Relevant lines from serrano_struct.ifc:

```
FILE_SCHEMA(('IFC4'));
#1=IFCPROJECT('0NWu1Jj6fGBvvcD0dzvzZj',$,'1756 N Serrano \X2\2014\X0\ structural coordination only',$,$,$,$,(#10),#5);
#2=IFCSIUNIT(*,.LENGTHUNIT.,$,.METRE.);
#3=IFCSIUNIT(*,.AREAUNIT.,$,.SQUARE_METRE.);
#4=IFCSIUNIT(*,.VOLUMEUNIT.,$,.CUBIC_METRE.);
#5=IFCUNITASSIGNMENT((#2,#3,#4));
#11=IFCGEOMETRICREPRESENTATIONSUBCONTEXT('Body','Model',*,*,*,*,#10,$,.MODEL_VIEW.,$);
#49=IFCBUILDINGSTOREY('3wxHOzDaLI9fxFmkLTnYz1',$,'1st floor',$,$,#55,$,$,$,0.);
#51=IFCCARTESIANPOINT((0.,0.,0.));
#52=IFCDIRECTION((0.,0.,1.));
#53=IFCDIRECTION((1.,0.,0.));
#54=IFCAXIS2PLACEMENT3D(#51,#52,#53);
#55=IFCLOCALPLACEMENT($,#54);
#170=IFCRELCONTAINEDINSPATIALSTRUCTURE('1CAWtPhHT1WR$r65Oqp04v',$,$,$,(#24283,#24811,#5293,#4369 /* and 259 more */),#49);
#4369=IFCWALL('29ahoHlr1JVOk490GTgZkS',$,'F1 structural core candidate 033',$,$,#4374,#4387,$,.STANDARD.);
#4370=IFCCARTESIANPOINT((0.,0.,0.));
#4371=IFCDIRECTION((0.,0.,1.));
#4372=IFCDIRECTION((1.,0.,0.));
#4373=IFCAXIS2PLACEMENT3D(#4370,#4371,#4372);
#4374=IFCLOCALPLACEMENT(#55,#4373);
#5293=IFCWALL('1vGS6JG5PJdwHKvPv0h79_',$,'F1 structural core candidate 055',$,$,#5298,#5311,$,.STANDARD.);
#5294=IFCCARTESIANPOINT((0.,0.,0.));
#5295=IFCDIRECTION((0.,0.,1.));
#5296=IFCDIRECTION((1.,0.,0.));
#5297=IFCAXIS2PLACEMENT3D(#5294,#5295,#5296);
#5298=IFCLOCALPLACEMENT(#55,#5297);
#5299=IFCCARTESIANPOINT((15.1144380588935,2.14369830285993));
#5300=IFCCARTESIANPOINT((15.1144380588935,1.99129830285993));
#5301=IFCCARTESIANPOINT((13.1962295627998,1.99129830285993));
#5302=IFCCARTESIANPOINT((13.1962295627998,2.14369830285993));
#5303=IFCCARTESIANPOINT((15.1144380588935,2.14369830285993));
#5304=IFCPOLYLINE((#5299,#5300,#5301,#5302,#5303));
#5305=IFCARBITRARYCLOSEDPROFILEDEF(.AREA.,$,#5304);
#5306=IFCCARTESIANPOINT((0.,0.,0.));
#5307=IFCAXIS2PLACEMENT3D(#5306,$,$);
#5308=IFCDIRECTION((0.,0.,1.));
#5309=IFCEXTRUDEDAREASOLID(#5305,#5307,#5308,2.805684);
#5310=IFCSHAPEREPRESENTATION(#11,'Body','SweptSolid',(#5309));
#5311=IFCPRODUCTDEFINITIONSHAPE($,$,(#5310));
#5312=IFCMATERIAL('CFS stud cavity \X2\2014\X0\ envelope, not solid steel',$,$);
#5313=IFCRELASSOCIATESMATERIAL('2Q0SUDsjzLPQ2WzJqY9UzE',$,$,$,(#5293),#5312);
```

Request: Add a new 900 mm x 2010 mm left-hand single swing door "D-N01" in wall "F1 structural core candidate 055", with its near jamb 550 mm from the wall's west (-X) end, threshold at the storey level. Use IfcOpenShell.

```python
import numpy as np
import ifcopenshell
import ifcopenshell.api.feature
import ifcopenshell.api.geometry
import ifcopenshell.api.root
import ifcopenshell.api.spatial
import ifcopenshell.geom
import ifcopenshell.util.element
import ifcopenshell.util.placement
import ifcopenshell.util.representation
import ifcopenshell.util.shape
import ifcopenshell.util.unit

model = ifcopenshell.open("serrano_struct.ifc")
unit_scale = ifcopenshell.util.unit.calculate_unit_scale(model)
settings = ifcopenshell.geom.settings()


def volume(element):
    """Net volume in cubic metres, openings subtracted."""
    shape = ifcopenshell.geom.create_shape(settings, element)
    return ifcopenshell.util.shape.get_volume(shape.geometry)


wall = model.by_id(5293)
storey = ifcopenshell.util.element.get_container(wall, ifc_class="IfcBuildingStorey")
context = ifcopenshell.util.representation.get_context(model, "Model", "Body", "MODEL_VIEW")
before = volume(wall)

width, height, from_end, sill = 0.9, 2.01, 0.55, 0.0  # metres

# The wall runs along its own X axis, and the end named is its -X end.
wall_shape = ifcopenshell.geom.create_shape(settings, wall)
x, y, z = ifcopenshell.util.shape.get_vertices(wall_shape.geometry).T
start = x.min() + from_end
face, thickness = float(y.min()), float(y.max() - y.min())
wall_matrix = ifcopenshell.util.placement.get_local_placement(wall.ObjectPlacement)
level = ifcopenshell.util.placement.get_local_placement(storey.ObjectPlacement)[2, 3]


def in_wall(x, y):
    """Placement at x, y metres in the wall's axes, at sill height."""
    matrix = wall_matrix.copy()
    matrix[:, 3] = wall_matrix @ np.array([x / unit_scale, y / unit_scale, 0.0, 1.0])
    matrix[2, 3] = level + sill / unit_scale
    return matrix


# Opening: a box that overshoots both wall faces by 50 mm.
opening = ifcopenshell.api.root.create_entity(model, ifc_class="IfcOpeningElement", predefined_type="OPENING")
box = ifcopenshell.api.geometry.add_wall_representation(
    model, context=context, length=width, height=height, thickness=thickness + 0.1
)
ifcopenshell.api.geometry.assign_representation(model, product=opening, representation=box)
ifcopenshell.api.geometry.edit_object_placement(model, product=opening, matrix=in_wall(start, face - 0.05), is_si=False)
ifcopenshell.api.feature.add_feature(model, feature=opening, element=wall)

door = ifcopenshell.api.root.create_entity(model, ifc_class="IfcDoor", name="D-N01", predefined_type="DOOR")
door.OverallWidth, door.OverallHeight = width / unit_scale, height / unit_scale
door.OperationType = "SINGLE_SWING_LEFT"
body = ifcopenshell.api.geometry.add_door_representation(
    model,
    context=context,
    overall_width=door.OverallWidth,
    overall_height=door.OverallHeight,
    operation_type="SINGLE_SWING_LEFT",
    lining_properties={"LiningDepth": thickness / unit_scale, "ThresholdDepth": thickness / unit_scale},
)
ifcopenshell.api.geometry.assign_representation(model, product=door, representation=body)
ifcopenshell.api.spatial.assign_container(model, products=[door], relating_structure=storey)
ifcopenshell.api.feature.add_filling(model, opening=opening, element=door)

# The lining spans the wall, so the door starts at the wall face.
ifcopenshell.api.geometry.edit_object_placement(model, product=door, matrix=in_wall(start, face), is_si=False)

after = volume(wall)

print(f"wall volume {before:.3f} -> {after:.3f} m3")

model.write("serrano_struct_updated.ifc")
```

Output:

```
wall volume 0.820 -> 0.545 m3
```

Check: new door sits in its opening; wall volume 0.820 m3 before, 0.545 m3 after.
